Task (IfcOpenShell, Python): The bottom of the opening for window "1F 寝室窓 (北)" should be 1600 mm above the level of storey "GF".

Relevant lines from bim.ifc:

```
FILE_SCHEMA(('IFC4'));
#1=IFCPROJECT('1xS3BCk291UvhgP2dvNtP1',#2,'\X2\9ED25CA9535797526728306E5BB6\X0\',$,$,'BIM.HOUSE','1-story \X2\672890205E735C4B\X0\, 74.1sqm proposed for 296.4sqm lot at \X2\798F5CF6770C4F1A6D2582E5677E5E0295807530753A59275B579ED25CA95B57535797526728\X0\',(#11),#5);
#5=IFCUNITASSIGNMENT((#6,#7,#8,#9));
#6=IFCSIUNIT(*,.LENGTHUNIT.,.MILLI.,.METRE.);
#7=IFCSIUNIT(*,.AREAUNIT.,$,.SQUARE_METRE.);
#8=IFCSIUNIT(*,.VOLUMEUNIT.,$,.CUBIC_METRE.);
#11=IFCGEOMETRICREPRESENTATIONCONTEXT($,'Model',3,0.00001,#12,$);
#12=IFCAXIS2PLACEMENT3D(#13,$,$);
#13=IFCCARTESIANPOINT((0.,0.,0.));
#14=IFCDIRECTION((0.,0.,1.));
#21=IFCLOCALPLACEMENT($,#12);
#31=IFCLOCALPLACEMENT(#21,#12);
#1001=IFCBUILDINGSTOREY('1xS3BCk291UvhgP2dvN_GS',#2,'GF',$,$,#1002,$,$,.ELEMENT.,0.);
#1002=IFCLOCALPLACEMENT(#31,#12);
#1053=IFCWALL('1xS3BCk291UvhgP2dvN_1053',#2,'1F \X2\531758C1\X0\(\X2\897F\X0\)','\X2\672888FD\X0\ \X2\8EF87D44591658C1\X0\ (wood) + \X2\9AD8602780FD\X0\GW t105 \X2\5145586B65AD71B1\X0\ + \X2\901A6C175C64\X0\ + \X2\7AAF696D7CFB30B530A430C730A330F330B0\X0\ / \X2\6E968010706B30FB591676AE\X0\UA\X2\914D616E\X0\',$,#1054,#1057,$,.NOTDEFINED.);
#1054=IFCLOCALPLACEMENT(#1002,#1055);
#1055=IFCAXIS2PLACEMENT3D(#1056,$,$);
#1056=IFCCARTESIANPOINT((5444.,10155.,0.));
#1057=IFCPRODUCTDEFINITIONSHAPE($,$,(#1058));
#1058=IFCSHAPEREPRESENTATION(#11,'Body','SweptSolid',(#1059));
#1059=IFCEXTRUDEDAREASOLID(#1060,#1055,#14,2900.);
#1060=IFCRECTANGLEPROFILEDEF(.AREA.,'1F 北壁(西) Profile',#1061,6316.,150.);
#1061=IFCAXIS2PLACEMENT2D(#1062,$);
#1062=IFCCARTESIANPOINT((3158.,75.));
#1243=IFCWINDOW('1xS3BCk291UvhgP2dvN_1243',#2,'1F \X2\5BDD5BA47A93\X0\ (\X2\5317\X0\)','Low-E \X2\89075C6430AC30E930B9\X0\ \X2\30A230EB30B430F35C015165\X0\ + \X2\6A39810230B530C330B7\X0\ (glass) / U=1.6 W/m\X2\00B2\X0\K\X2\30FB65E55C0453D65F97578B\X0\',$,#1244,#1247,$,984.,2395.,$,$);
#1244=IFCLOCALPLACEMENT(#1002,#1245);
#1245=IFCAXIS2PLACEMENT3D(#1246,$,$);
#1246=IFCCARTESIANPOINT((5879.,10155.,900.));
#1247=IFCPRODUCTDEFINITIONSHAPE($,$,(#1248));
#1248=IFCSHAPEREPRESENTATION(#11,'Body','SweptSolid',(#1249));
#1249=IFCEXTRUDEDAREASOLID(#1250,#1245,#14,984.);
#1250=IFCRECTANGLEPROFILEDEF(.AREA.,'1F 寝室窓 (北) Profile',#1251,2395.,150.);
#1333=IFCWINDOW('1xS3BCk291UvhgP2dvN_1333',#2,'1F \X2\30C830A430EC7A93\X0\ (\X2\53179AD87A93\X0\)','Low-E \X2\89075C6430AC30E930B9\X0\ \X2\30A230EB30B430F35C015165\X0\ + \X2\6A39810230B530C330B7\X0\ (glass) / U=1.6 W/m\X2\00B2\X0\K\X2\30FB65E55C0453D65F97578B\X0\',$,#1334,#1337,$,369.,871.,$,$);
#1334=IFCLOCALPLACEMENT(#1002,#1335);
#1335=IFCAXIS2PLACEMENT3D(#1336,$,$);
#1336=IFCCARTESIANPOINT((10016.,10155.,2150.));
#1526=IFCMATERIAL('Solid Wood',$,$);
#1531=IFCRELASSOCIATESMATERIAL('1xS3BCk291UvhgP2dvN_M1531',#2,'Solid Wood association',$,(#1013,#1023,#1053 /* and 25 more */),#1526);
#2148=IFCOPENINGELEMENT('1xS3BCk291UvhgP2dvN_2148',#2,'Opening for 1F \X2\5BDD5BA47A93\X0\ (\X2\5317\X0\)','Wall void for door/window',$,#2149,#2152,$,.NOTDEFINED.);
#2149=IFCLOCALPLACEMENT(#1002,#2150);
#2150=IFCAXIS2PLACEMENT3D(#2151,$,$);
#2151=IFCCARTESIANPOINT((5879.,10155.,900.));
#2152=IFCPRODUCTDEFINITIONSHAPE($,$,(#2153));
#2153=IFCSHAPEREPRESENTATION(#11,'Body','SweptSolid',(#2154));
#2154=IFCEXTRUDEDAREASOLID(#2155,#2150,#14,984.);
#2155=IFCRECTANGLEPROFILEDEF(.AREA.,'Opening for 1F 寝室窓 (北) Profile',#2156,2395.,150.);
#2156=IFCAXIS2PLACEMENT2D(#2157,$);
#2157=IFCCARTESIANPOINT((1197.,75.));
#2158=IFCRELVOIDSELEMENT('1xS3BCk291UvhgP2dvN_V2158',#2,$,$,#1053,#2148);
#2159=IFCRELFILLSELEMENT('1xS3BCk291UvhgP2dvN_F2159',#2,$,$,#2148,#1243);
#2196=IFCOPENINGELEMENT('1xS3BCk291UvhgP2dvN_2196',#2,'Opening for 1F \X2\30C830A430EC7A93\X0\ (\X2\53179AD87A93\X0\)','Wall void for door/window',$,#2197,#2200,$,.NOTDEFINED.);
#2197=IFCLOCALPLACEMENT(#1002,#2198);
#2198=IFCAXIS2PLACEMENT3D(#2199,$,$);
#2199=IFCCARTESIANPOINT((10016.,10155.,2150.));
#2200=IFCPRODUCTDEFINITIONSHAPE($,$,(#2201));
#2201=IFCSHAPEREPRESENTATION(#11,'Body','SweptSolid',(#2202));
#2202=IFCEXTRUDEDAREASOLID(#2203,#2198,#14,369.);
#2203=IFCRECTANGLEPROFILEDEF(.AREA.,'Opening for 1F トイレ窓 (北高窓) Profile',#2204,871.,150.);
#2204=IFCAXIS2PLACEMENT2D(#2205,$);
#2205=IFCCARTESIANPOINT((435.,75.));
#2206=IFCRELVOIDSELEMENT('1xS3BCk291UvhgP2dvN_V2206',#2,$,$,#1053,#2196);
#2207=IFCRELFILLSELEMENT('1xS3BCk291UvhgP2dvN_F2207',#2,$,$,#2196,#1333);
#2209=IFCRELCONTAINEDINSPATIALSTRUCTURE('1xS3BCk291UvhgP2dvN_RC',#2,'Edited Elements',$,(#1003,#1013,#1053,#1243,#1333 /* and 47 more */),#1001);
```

```python
import numpy as np
import ifcopenshell
import ifcopenshell.api.geometry
import ifcopenshell.geom
import ifcopenshell.util.element
import ifcopenshell.util.placement
import ifcopenshell.util.shape
import ifcopenshell.util.unit

model = ifcopenshell.open("bim.ifc")
unit_scale = ifcopenshell.util.unit.calculate_unit_scale(model)

window = model.by_guid("1xS3BCk291UvhgP2dvN_1243")
opening = window.FillsVoids[0].RelatingOpeningElement
storey = ifcopenshell.util.element.get_container(window, ifc_class="IfcBuildingStorey")
level = ifcopenshell.util.placement.get_local_placement(storey.ObjectPlacement)[2, 3]

# The opening's origin need not be at the sill, so measure its lowest point.
shape = ifcopenshell.geom.create_shape(ifcopenshell.geom.settings(), opening)
bottom = ifcopenshell.util.shape.get_shape_bottom_elevation(shape, shape.geometry) / unit_scale
dz = level + 1.6 / unit_scale - bottom

shift = np.array([0.0, 0.0, dz])
# The window is not placed relative to its opening, so move both.
for product in (opening, window):
    matrix = ifcopenshell.util.placement.get_local_placement(product.ObjectPlacement)
    matrix[:3, 3] += shift
    ifcopenshell.api.geometry.edit_object_placement(model, product=product, matrix=matrix, is_si=False)

print(f"moved by {dz * unit_scale:+.3f} m")

model.write("bim_updated.ifc")
```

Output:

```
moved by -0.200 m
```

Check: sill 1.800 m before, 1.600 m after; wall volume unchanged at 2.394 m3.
